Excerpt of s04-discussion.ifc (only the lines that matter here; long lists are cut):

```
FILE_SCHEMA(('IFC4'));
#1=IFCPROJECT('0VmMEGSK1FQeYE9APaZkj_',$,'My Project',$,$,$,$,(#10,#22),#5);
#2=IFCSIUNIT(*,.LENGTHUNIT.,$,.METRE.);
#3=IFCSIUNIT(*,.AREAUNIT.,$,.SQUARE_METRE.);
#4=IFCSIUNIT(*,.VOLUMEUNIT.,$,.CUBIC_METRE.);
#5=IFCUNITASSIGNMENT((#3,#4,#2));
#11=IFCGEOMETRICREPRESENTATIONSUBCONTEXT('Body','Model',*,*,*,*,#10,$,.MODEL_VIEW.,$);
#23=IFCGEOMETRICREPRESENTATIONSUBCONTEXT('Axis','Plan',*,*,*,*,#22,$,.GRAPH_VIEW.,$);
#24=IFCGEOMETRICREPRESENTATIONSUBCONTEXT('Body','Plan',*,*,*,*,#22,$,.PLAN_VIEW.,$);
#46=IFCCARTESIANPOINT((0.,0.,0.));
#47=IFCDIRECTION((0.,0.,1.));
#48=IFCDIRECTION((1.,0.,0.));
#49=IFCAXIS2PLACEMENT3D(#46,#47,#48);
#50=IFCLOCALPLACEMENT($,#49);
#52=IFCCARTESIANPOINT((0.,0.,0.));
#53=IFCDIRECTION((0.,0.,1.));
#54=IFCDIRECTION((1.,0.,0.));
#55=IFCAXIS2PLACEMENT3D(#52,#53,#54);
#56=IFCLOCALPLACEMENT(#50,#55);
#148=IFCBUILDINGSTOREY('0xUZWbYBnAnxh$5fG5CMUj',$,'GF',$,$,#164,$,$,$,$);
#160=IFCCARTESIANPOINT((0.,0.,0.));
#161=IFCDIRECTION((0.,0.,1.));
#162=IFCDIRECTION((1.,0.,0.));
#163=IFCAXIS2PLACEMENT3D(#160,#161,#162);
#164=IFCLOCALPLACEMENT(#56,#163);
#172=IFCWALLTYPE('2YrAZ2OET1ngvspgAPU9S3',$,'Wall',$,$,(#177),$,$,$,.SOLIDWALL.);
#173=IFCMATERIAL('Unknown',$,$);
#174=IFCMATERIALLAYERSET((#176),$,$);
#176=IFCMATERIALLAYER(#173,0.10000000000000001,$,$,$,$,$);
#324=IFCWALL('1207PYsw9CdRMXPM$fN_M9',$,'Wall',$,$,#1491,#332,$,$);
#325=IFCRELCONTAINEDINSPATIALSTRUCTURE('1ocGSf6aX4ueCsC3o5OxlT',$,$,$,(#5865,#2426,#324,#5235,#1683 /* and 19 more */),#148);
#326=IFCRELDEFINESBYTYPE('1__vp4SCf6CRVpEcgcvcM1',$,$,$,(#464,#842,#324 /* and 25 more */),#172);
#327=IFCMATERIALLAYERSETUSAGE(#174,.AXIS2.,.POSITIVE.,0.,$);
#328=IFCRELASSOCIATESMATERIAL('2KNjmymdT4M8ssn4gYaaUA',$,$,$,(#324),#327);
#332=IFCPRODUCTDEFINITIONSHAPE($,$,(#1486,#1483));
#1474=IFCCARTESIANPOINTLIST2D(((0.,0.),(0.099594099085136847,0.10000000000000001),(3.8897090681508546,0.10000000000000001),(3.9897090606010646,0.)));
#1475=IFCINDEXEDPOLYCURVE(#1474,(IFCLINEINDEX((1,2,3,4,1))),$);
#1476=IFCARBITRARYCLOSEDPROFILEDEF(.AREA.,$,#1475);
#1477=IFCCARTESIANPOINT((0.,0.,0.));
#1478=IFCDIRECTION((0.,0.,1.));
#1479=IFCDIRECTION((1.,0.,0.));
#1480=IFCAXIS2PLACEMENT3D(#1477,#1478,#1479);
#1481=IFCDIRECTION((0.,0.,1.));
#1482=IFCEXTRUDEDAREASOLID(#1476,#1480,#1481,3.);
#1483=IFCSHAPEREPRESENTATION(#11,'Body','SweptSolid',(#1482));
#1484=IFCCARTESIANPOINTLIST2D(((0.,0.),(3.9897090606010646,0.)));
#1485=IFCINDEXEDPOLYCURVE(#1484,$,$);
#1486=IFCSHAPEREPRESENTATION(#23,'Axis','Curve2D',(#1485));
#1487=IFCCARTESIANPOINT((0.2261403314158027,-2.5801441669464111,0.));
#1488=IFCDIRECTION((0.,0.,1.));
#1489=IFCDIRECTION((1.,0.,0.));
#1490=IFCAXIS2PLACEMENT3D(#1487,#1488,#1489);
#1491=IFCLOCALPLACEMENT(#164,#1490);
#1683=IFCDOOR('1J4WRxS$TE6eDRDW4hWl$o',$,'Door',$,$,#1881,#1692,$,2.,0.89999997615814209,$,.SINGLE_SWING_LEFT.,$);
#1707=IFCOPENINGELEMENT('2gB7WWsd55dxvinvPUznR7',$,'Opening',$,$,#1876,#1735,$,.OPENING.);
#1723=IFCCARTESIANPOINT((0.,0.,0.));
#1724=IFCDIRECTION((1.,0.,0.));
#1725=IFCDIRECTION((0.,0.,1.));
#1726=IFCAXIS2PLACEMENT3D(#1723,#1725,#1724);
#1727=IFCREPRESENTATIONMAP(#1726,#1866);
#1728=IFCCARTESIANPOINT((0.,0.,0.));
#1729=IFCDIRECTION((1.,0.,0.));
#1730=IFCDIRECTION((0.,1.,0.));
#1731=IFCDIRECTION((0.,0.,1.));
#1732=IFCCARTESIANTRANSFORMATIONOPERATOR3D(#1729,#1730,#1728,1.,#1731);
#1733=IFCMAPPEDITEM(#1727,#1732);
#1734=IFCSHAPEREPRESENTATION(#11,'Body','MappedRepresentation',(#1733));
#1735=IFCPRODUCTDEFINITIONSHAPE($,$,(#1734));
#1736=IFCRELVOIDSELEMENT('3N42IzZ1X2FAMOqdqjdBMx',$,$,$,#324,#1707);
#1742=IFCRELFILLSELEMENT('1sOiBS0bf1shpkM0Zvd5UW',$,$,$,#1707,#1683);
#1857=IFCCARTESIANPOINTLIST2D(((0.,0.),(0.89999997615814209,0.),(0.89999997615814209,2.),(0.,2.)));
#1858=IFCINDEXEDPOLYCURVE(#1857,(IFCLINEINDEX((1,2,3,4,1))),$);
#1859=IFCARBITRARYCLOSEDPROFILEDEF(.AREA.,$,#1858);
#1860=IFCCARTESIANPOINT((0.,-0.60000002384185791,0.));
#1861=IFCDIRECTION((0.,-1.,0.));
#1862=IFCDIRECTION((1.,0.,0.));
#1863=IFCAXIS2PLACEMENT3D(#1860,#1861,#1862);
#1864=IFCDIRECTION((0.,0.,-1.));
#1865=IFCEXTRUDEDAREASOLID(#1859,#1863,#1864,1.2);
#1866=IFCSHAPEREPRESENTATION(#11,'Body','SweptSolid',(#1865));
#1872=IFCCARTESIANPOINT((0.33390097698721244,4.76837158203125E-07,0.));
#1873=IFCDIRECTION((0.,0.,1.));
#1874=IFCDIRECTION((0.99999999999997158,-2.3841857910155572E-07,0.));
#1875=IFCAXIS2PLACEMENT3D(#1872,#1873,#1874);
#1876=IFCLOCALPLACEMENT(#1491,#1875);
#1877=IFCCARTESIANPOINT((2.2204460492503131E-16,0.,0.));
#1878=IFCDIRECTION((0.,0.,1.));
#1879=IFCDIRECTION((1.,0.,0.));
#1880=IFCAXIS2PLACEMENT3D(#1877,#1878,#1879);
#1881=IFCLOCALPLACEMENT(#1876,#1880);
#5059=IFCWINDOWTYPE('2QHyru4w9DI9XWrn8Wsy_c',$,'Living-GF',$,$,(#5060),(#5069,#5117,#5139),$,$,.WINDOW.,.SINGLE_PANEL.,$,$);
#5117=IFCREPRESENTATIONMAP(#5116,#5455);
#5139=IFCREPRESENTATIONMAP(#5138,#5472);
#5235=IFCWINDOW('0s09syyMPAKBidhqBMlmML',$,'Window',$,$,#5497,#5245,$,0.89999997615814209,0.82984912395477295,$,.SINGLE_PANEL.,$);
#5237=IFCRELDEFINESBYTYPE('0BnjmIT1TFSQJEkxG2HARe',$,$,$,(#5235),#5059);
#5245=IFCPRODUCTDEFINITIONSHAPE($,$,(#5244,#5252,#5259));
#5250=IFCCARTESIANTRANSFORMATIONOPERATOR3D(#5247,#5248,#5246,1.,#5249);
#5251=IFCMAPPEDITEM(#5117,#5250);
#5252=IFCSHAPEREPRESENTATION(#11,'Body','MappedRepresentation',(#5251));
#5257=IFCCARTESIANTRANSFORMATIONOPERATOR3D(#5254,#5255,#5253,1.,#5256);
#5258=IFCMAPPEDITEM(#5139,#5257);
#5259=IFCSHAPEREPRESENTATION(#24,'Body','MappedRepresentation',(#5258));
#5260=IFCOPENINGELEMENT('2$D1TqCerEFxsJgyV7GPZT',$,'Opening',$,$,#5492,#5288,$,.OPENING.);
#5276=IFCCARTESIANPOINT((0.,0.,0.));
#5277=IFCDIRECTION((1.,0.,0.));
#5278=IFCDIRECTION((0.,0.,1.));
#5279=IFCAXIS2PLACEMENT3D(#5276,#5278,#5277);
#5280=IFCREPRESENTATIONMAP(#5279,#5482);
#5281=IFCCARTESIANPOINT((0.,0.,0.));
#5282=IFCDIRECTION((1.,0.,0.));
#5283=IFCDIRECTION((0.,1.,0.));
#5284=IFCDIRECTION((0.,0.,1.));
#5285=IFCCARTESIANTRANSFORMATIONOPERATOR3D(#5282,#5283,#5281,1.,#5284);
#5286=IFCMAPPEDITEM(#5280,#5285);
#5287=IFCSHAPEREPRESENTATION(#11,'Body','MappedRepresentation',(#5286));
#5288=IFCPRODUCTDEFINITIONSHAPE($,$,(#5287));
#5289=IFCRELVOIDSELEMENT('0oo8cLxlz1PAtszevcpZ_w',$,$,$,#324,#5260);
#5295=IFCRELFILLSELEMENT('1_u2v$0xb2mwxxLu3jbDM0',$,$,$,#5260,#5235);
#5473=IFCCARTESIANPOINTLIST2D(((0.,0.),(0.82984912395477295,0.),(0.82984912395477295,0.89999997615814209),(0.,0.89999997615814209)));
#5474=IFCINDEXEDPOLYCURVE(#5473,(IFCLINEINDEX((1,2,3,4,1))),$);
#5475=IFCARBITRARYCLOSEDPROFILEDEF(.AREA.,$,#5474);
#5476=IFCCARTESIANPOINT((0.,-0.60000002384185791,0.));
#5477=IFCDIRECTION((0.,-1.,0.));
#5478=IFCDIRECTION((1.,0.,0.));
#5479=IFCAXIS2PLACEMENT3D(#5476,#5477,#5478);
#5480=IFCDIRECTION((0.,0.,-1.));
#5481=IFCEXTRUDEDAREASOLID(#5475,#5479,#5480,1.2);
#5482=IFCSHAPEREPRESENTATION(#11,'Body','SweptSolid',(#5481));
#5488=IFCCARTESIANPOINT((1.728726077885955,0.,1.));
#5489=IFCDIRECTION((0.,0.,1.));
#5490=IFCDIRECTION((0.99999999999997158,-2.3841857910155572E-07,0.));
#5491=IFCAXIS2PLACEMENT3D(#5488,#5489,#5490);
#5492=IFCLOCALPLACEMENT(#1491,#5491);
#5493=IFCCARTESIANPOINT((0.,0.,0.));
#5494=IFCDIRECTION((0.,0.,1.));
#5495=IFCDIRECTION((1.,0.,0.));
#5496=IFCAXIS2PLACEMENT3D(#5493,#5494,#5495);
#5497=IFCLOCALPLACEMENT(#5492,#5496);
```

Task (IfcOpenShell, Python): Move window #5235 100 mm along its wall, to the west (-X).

```python
import ifcopenshell
import ifcopenshell.api.geometry
import ifcopenshell.util.placement
import ifcopenshell.util.unit

model = ifcopenshell.open("s04-discussion.ifc")
unit_scale = ifcopenshell.util.unit.calculate_unit_scale(model)

window = model.by_guid("0s09syyMPAKBidhqBMlmML")
opening = window.FillsVoids[0].RelatingOpeningElement
wall = opening.VoidsElements[0].RelatingBuildingElement

wall_matrix = ifcopenshell.util.placement.get_local_placement(wall.ObjectPlacement)
shift = wall_matrix[:3, 0] * -0.1 / unit_scale
before = ifcopenshell.util.placement.get_local_placement(window.ObjectPlacement)[:3, 3].copy()

# The window is placed relative to its opening, so it follows when the opening moves.
matrix = ifcopenshell.util.placement.get_local_placement(opening.ObjectPlacement)
matrix[:3, 3] += shift
ifcopenshell.api.geometry.edit_object_placement(
    model, product=opening, matrix=matrix, is_si=False, should_transform_children=True
)

after = ifcopenshell.util.placement.get_local_placement(window.ObjectPlacement)[:3, 3]
print("window moved by", (after - before).round(3) + 0.0)

model.write("s04-discussion_edited.ifc")
```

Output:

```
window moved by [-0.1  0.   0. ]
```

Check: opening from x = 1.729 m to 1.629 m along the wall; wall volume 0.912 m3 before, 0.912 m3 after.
